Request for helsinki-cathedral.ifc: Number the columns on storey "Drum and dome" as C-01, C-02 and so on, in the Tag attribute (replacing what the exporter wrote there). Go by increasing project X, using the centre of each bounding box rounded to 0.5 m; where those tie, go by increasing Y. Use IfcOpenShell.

First a look at what the model holds.

```python
import ifcopenshell
import ifcopenshell.util.element
import ifcopenshell.util.placement

model = ifcopenshell.open("helsinki-cathedral.ifc")
print(model.schema)
storey = next(s for s in model.by_type("IfcBuildingStorey") if s.Name == "Drum and dome")
columns = [e for e in ifcopenshell.util.element.get_decomposition(storey) if e.is_a("IfcColumn")]
for e in sorted(columns, key=lambda e: e.id()):
    origin = ifcopenshell.util.placement.get_local_placement(e.ObjectPlacement)[:3, 3]
    print(e.id(), e.Tag, e.Name, origin.round(2) + 0.0, sep=" | ")
```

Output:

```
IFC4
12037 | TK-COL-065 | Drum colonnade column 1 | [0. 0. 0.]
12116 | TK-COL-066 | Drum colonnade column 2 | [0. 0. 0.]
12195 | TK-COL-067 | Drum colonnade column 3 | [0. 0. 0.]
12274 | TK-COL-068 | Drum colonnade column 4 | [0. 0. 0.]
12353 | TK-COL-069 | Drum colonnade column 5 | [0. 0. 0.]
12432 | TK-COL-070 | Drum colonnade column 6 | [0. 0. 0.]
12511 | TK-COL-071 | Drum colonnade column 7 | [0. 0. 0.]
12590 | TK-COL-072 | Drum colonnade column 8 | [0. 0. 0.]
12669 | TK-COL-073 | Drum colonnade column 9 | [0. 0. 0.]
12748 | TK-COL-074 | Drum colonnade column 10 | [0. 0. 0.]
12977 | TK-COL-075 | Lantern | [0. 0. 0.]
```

```python
import ifcopenshell
import ifcopenshell.geom
import ifcopenshell.util.element
import ifcopenshell.util.shape

model = ifcopenshell.open("helsinki-cathedral.ifc")
settings = ifcopenshell.geom.settings()
settings.set("use-world-coords", True)


def centre(element):
    shape = ifcopenshell.geom.create_shape(settings, element)
    return ifcopenshell.util.shape.get_bbox_centroid(shape.geometry)


storey = next(s for s in model.by_type("IfcBuildingStorey") if s.Name == "Drum and dome")
columns = [e for e in ifcopenshell.util.element.get_decomposition(storey) if e.is_a("IfcColumn")]

# Insertion points can sit at a corner or the storey origin, so sort by the geometry (in metres).
centres = {e: centre(e) for e in columns}
columns.sort(key=lambda e: (round(centres[e][0] / 0.5), centres[e][1]))

for i, e in enumerate(columns, start=1):
    number = f"C-{i:02d}"
    e.Tag = number
    print(e.id(), number)

model.write("helsinki-cathedral_edited.ifc")
```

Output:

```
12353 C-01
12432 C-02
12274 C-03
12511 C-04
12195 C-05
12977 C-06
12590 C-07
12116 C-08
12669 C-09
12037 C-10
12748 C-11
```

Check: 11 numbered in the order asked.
